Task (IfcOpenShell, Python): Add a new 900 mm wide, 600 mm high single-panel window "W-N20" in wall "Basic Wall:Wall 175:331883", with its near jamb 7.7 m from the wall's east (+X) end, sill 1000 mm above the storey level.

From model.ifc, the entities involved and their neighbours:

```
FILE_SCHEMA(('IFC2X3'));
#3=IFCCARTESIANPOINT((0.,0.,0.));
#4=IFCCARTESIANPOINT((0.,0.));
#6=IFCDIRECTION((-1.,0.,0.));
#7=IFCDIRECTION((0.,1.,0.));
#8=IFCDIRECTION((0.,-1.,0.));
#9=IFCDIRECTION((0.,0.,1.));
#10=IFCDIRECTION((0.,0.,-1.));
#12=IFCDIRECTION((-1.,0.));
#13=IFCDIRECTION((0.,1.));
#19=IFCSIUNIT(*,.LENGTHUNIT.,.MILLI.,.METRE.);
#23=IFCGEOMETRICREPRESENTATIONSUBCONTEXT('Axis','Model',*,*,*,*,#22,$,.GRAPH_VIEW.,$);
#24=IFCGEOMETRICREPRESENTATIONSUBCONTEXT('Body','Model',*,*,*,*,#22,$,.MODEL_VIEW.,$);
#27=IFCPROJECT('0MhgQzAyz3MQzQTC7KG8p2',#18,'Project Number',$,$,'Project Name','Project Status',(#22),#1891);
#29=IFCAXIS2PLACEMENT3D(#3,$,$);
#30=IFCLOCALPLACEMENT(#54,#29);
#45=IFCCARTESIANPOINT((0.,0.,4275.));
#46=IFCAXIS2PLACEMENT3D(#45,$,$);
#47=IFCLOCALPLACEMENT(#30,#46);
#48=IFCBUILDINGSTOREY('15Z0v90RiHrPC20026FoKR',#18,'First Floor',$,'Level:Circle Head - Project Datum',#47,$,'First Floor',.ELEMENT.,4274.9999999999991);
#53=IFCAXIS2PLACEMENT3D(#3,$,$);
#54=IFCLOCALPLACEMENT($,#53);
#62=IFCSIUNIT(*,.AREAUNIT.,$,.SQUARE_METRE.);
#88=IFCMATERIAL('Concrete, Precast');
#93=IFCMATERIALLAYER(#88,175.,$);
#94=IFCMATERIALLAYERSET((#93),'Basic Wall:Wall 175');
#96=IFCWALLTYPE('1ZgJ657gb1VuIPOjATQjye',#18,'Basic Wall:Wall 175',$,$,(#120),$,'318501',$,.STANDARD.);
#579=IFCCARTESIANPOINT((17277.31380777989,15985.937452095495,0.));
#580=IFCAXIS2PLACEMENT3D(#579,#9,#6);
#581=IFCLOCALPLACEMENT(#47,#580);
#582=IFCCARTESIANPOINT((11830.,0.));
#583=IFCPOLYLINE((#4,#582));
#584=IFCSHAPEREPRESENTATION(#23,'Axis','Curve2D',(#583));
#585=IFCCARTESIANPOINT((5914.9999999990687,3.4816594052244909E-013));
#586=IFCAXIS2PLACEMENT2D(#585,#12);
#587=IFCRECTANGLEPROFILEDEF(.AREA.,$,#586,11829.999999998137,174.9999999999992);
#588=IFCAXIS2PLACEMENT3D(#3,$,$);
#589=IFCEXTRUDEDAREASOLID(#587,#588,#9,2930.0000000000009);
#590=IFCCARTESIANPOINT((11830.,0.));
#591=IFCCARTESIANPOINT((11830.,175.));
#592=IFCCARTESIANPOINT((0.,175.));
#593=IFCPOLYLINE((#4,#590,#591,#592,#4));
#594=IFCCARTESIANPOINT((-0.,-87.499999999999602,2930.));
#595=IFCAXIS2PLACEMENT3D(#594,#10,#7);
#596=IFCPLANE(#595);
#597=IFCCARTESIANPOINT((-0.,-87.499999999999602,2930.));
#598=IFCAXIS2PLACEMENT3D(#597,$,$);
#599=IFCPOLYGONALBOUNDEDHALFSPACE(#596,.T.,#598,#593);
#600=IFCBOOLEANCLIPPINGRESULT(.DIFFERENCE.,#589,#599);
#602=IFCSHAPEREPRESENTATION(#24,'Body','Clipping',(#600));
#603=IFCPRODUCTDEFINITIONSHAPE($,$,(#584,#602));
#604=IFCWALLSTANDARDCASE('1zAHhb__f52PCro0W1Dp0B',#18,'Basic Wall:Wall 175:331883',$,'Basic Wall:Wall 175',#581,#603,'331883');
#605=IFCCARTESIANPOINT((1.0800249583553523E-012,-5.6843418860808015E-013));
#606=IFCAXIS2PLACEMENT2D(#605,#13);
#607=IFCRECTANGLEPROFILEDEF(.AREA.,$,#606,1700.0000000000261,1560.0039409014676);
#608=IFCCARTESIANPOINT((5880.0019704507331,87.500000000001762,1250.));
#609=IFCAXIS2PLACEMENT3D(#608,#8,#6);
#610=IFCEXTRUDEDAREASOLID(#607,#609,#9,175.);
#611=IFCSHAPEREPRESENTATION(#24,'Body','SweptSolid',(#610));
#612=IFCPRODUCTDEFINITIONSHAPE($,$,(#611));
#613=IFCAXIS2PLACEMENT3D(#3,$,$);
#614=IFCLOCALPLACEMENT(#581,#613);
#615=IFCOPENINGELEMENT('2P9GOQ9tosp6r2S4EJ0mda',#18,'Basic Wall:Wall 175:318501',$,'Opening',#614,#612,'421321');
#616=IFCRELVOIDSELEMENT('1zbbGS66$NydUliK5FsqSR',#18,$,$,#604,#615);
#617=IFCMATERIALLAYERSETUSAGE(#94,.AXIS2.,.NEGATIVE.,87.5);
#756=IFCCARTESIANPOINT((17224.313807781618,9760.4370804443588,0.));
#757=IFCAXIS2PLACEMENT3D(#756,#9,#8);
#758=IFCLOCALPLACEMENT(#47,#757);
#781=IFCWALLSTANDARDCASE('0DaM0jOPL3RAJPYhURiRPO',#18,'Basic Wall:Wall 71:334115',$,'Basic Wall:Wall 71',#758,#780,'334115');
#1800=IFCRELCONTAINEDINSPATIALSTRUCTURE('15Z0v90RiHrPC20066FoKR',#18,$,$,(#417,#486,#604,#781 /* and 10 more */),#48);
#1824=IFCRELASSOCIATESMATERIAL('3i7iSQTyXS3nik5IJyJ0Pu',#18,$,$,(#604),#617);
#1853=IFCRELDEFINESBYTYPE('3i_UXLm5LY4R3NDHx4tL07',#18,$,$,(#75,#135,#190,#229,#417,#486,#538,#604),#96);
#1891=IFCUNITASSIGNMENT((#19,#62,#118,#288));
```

```python
import numpy as np
import ifcopenshell
import ifcopenshell.api.feature
import ifcopenshell.api.geometry
import ifcopenshell.api.root
import ifcopenshell.api.spatial
import ifcopenshell.api.type
import ifcopenshell.geom
import ifcopenshell.util.element
import ifcopenshell.util.placement
import ifcopenshell.util.representation
import ifcopenshell.util.shape
import ifcopenshell.util.unit

model = ifcopenshell.open("model.ifc")
unit_scale = ifcopenshell.util.unit.calculate_unit_scale(model)
settings = ifcopenshell.geom.settings()


def volume(element):
    """Net volume in cubic metres, openings subtracted."""
    shape = ifcopenshell.geom.create_shape(settings, element)
    return ifcopenshell.util.shape.get_volume(shape.geometry)


wall = model.by_id(604)
storey = ifcopenshell.util.element.get_container(wall, ifc_class="IfcBuildingStorey")
context = ifcopenshell.util.representation.get_context(model, "Model", "Body", "MODEL_VIEW")
before = volume(wall)

width, height, from_end, sill = 0.9, 0.6, 7.7, 1  # metres

# The wall runs along its own X axis, and the end named is its -X end.
wall_shape = ifcopenshell.geom.create_shape(settings, wall)
x, y, z = ifcopenshell.util.shape.get_vertices(wall_shape.geometry).T
start = x.min() + from_end
face, thickness = float(y.min()), float(y.max() - y.min())
wall_matrix = ifcopenshell.util.placement.get_local_placement(wall.ObjectPlacement)
level = ifcopenshell.util.placement.get_local_placement(storey.ObjectPlacement)[2, 3]


def in_wall(x, y):
    """Placement at x, y metres in the wall's axes, at sill height."""
    matrix = wall_matrix.copy()
    matrix[:, 3] = wall_matrix @ np.array([x / unit_scale, y / unit_scale, 0.0, 1.0])
    matrix[2, 3] = level + sill / unit_scale
    return matrix


# Opening: a box that overshoots both wall faces by 50 mm.
opening = ifcopenshell.api.root.create_entity(model, ifc_class="IfcOpeningElement")
box = ifcopenshell.api.geometry.add_wall_representation(
    model, context=context, length=width, height=height, thickness=thickness + 0.1
)
ifcopenshell.api.geometry.assign_representation(model, product=opening, representation=box)
ifcopenshell.api.geometry.edit_object_placement(model, product=opening, matrix=in_wall(start, face - 0.05), is_si=False)
ifcopenshell.api.feature.add_feature(model, feature=opening, element=wall)

window = ifcopenshell.api.root.create_entity(model, ifc_class="IfcWindow", name="W-N20")
window.OverallWidth, window.OverallHeight = width / unit_scale, height / unit_scale
body = ifcopenshell.api.geometry.add_window_representation(
    model,
    context=context,
    overall_width=window.OverallWidth,
    overall_height=window.OverallHeight,
    partition_type="SINGLE_PANEL",
)
ifcopenshell.api.geometry.assign_representation(model, product=window, representation=body)
ifcopenshell.api.spatial.assign_container(model, products=[window], relating_structure=storey)
fills = ifcopenshell.api.feature.add_filling(model, opening=opening, element=window)
fills.OwnerHistory = window.OwnerHistory  # required in IFC2X3

# IFC2X3 keeps the operation on the window style.
style = ifcopenshell.api.root.create_entity(model, ifc_class="IfcWindowStyle", name="W-N20")
style.OperationType, style.ConstructionType = "SINGLE_PANEL", "NOTDEFINED"
style.ParameterTakesPrecedence = style.Sizeable = False
ifcopenshell.api.type.assign_type(model, related_objects=[window], relating_type=style)

# Centre the window in the wall's thickness.
ifcopenshell.api.geometry.edit_object_placement(model, product=window, matrix=in_wall(start, face), is_si=False)
window_shape = ifcopenshell.geom.create_shape(settings, window)
depth = ifcopenshell.util.shape.get_vertices(window_shape.geometry)[:, 1]
offset = face + thickness / 2 - (depth.min() + depth.max()) / 2
ifcopenshell.api.geometry.edit_object_placement(model, product=window, matrix=in_wall(start, offset), is_si=False)

after = volume(wall)

print(f"wall volume {before:.3f} -> {after:.3f} m3")

model.write("model_edited.ifc")
```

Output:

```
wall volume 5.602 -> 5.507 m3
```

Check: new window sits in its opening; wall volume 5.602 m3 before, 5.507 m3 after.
